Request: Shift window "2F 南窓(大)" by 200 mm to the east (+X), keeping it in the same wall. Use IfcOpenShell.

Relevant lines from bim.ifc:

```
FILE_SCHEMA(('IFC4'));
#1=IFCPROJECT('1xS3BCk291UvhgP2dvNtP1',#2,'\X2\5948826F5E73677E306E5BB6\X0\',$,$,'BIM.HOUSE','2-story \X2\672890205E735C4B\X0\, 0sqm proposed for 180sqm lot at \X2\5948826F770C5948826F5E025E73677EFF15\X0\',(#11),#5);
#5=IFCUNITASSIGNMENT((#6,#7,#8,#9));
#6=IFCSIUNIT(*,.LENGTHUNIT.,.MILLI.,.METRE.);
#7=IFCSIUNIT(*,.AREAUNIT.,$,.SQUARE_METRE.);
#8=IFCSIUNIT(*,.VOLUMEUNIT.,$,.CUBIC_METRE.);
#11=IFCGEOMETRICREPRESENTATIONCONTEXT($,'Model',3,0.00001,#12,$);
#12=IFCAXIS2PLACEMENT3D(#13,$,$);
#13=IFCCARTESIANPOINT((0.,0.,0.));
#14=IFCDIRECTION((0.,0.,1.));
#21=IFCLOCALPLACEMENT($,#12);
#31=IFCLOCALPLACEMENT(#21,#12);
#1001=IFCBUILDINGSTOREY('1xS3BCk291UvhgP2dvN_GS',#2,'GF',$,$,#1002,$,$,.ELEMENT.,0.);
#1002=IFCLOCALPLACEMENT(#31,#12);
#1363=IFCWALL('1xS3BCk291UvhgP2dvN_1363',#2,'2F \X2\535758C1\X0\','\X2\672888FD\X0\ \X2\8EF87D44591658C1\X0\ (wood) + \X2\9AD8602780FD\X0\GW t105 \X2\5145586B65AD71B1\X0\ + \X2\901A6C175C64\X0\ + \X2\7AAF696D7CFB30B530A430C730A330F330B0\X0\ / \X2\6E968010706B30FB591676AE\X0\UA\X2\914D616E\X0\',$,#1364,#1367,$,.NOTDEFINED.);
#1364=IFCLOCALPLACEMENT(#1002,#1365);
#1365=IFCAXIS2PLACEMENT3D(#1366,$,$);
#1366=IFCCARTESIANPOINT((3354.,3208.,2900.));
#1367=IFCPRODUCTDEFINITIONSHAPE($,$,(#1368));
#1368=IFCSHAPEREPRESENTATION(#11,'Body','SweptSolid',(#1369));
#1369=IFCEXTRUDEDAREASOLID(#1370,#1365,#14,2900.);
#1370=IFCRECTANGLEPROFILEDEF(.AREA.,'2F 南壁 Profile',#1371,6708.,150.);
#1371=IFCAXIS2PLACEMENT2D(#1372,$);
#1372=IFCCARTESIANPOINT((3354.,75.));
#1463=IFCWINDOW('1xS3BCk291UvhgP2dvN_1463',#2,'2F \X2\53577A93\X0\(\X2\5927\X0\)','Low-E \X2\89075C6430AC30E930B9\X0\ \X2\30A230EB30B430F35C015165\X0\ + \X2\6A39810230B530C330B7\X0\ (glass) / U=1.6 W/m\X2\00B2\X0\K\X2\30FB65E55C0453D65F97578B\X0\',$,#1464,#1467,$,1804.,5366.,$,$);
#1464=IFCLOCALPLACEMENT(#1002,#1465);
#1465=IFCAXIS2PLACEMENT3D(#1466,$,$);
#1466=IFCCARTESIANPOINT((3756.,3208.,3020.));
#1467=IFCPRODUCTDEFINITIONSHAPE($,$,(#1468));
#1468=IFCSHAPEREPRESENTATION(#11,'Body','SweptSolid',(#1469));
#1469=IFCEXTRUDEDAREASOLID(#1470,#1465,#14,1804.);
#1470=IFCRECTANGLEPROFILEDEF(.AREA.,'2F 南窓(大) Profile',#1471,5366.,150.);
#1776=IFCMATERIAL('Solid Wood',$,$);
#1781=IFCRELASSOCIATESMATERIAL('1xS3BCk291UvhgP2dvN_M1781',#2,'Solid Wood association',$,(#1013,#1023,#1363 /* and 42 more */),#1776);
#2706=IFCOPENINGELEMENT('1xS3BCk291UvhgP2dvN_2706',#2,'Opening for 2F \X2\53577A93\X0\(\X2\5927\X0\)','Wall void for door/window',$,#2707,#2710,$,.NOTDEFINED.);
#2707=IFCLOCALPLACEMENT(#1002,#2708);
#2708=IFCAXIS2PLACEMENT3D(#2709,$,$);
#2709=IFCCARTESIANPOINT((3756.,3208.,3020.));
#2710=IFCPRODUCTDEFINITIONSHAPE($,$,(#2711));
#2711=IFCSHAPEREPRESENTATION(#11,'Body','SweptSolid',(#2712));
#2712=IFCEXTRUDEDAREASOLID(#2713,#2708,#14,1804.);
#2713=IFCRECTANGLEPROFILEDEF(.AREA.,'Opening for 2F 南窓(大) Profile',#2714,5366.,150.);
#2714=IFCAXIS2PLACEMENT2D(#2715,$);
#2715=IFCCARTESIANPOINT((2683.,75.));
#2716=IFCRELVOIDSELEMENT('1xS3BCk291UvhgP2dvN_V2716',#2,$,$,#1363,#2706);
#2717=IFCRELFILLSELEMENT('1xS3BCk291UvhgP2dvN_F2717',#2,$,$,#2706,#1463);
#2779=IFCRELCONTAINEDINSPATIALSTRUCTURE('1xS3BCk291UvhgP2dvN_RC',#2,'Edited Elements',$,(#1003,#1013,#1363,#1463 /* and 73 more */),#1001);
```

```python
import ifcopenshell
import ifcopenshell.api.geometry
import ifcopenshell.util.placement

model = ifcopenshell.open("bim.ifc")

window = model.by_id(1463)
opening = window.FillsVoids[0].RelatingOpeningElement
wall = opening.VoidsElements[0].RelatingBuildingElement

wall_matrix = ifcopenshell.util.placement.get_local_placement(wall.ObjectPlacement)
shift = wall_matrix[:3, 0] * 200.0
before = ifcopenshell.util.placement.get_local_placement(window.ObjectPlacement)[:3, 3].copy()

# The window is not placed relative to its opening, so move both.
for product in (opening, window):
    matrix = ifcopenshell.util.placement.get_local_placement(product.ObjectPlacement)
    matrix[:3, 3] += shift
    ifcopenshell.api.geometry.edit_object_placement(model, product=product, matrix=matrix, is_si=False)

after = ifcopenshell.util.placement.get_local_placement(window.ObjectPlacement)[:3, 3]
print("window moved by", (after - before).round(3) + 0.0)

model.write("bim-out.ifc")
```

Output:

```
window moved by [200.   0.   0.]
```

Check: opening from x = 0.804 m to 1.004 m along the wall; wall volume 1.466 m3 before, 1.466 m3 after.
